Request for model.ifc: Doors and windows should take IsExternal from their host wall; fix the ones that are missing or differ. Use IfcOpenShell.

First a look at what the model holds.

```python
import ifcopenshell
import ifcopenshell.util.element

model = ifcopenshell.open("model.ifc")
print(model.schema)
seen = {}
for e in model.by_type("IfcDoor") + model.by_type("IfcWindow"):
    if not e.FillsVoids:
        continue
    host = e.FillsVoids[0].RelatingOpeningElement.VoidsElements[0].RelatingBuildingElement
    own = ifcopenshell.util.element.get_pset(e, f"Pset_{e.is_a()[3:].removesuffix('StandardCase')}Common", "IsExternal")
    wall = ifcopenshell.util.element.get_pset(host, "Pset_WallCommon", "IsExternal")
    seen[e.is_a(), own, wall] = seen.get((e.is_a(), own, wall), 0) + 1
for (cls, own, wall), count in sorted(seen.items(), key=str):
    print(count, cls, "IsExternal:", own, "| host wall:", wall)
```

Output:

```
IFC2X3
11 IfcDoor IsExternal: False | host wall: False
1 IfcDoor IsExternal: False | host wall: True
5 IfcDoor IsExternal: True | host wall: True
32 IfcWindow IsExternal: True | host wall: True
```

```python
import ifcopenshell
import ifcopenshell.api.pset
import ifcopenshell.util.element

model = ifcopenshell.open("model.ifc")

count = 0
for ifc_class, pset_name in (("IfcDoor", "Pset_DoorCommon"), ("IfcWindow", "Pset_WindowCommon")):
    for e in model.by_type(ifc_class):
        if not e.FillsVoids:
            continue
        host = e.FillsVoids[0].RelatingOpeningElement.VoidsElements[0].RelatingBuildingElement
        external = ifcopenshell.util.element.get_pset(host, "Pset_WallCommon", "IsExternal")
        if external is None or ifcopenshell.util.element.get_pset(e, pset_name, "IsExternal") == external:
            continue
        pset = ifcopenshell.api.pset.add_pset(model, product=e, name=pset_name)
        ifcopenshell.api.pset.edit_pset(model, pset=pset, properties={"IsExternal": external})
        count += 1

print(count, "updated")

model.write("model_v2.ifc")
```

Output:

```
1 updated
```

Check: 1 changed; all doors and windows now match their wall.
